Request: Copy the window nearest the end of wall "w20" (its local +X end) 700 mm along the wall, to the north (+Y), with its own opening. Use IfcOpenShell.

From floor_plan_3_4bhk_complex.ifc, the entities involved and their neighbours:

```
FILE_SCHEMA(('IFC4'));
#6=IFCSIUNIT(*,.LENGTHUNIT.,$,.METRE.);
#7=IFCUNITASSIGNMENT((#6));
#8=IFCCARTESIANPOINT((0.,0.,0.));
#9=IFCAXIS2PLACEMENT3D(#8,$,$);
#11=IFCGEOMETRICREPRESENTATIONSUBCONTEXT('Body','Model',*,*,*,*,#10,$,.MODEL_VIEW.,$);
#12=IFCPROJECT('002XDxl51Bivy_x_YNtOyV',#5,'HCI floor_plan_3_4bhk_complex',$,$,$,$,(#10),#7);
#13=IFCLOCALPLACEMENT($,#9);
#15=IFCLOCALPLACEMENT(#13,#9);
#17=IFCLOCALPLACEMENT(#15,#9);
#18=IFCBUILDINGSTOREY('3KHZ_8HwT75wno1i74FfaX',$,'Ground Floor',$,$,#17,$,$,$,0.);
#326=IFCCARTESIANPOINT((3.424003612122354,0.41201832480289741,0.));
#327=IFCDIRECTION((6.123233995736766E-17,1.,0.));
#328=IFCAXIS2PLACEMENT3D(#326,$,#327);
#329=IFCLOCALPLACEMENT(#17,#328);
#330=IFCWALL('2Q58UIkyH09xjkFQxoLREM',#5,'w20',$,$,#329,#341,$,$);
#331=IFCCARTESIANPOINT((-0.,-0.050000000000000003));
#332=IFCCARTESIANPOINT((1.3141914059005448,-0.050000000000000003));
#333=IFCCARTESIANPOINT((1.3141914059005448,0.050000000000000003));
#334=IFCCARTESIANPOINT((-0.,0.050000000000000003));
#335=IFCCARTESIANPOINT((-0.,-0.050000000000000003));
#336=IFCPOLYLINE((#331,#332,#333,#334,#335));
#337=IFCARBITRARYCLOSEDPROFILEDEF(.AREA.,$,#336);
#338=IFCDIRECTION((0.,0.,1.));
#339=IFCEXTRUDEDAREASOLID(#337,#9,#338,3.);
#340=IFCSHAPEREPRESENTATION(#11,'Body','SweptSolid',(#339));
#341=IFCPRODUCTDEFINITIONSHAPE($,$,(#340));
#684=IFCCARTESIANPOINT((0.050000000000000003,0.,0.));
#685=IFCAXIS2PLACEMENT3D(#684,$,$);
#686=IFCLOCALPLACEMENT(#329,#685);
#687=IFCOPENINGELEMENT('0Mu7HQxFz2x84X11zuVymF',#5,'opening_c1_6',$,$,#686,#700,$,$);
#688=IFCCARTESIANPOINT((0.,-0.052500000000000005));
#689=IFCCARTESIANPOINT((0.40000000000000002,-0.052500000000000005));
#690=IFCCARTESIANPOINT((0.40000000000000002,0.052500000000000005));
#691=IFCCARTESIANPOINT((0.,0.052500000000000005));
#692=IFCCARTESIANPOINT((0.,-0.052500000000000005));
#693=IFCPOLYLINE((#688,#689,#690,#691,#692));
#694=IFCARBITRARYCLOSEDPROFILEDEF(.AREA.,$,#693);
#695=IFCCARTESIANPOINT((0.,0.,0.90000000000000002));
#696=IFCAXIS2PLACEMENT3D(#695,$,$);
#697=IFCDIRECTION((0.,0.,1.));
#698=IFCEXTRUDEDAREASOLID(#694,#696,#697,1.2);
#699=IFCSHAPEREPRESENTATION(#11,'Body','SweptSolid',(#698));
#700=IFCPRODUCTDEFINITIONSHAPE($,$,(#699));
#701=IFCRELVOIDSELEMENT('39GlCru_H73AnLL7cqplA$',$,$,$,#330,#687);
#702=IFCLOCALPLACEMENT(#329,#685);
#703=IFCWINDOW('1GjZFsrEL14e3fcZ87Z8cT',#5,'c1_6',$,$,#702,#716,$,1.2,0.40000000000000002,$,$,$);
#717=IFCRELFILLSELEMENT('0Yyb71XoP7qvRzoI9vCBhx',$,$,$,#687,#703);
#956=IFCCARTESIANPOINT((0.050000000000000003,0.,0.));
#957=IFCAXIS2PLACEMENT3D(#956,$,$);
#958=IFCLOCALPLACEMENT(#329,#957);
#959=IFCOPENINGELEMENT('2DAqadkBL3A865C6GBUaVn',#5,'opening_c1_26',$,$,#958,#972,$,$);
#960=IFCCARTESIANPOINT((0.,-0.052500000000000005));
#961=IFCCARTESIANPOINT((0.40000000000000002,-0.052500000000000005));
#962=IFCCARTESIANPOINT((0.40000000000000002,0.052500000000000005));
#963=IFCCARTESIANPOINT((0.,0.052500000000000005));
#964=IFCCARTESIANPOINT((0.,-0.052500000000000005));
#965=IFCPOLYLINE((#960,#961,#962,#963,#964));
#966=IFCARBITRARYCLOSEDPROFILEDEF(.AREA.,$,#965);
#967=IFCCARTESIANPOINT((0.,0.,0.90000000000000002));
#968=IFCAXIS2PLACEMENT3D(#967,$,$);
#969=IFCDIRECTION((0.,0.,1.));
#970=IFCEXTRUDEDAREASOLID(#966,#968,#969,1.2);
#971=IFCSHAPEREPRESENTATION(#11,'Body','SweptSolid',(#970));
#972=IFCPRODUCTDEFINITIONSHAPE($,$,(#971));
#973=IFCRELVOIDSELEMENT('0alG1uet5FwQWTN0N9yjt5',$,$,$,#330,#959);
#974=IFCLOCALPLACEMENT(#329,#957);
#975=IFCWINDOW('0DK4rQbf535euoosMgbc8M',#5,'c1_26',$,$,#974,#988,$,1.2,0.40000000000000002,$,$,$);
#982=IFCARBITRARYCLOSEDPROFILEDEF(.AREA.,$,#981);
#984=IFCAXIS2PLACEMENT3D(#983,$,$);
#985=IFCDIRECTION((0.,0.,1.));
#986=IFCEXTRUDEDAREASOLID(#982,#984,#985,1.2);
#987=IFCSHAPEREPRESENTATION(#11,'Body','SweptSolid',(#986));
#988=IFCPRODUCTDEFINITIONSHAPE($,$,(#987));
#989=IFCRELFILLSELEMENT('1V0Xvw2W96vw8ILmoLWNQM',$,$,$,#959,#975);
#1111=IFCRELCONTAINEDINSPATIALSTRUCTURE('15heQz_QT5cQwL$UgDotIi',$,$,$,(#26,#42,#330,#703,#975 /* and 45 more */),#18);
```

```python
import ifcopenshell
import ifcopenshell.api.feature
import ifcopenshell.api.geometry
import ifcopenshell.api.root
import ifcopenshell.geom
import ifcopenshell.util.element
import ifcopenshell.util.placement
import ifcopenshell.util.shape
import ifcopenshell.util.unit

model = ifcopenshell.open("floor_plan_3_4bhk_complex.ifc")
unit_scale = ifcopenshell.util.unit.calculate_unit_scale(model)
settings = ifcopenshell.geom.settings()


def volume(element):
    """Net volume in cubic metres, openings subtracted."""
    shape = ifcopenshell.geom.create_shape(settings, element)
    return ifcopenshell.util.shape.get_volume(shape.geometry)


window = model.by_guid("0DK4rQbf535euoosMgbc8M")
opening = window.FillsVoids[0].RelatingOpeningElement
wall = opening.VoidsElements[0].RelatingBuildingElement
before = volume(wall)
shift = ifcopenshell.util.placement.get_local_placement(wall.ObjectPlacement)[:3, 0] * 0.7 / unit_scale

# copy_class copies the void relationship, type, container and properties, but no geometry.
new_opening = ifcopenshell.api.root.copy_class(model, product=opening)
new_opening.Representation = ifcopenshell.util.element.copy_deep(
    model, opening.Representation, exclude=["IfcGeometricRepresentationContext", "IfcRepresentationMap"]
)
new_window = ifcopenshell.api.root.copy_class(model, product=window)
new_window.Representation = ifcopenshell.util.element.copy_deep(
    model, window.Representation, exclude=["IfcGeometricRepresentationContext", "IfcRepresentationMap"]
)
ifcopenshell.api.feature.add_filling(model, opening=new_opening, element=new_window)

for old, new in ((opening, new_opening), (window, new_window)):
    matrix = ifcopenshell.util.placement.get_local_placement(old.ObjectPlacement)
    matrix[:3, 3] += shift
    ifcopenshell.api.geometry.edit_object_placement(model, product=new, matrix=matrix, is_si=False)

after = volume(wall)

print(f"wall volume {before:.3f} -> {after:.3f} m3")

model.write("floor_plan_3_4bhk_complex-out.ifc")
```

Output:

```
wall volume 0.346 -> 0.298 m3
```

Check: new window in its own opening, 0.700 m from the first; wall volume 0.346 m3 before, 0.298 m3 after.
